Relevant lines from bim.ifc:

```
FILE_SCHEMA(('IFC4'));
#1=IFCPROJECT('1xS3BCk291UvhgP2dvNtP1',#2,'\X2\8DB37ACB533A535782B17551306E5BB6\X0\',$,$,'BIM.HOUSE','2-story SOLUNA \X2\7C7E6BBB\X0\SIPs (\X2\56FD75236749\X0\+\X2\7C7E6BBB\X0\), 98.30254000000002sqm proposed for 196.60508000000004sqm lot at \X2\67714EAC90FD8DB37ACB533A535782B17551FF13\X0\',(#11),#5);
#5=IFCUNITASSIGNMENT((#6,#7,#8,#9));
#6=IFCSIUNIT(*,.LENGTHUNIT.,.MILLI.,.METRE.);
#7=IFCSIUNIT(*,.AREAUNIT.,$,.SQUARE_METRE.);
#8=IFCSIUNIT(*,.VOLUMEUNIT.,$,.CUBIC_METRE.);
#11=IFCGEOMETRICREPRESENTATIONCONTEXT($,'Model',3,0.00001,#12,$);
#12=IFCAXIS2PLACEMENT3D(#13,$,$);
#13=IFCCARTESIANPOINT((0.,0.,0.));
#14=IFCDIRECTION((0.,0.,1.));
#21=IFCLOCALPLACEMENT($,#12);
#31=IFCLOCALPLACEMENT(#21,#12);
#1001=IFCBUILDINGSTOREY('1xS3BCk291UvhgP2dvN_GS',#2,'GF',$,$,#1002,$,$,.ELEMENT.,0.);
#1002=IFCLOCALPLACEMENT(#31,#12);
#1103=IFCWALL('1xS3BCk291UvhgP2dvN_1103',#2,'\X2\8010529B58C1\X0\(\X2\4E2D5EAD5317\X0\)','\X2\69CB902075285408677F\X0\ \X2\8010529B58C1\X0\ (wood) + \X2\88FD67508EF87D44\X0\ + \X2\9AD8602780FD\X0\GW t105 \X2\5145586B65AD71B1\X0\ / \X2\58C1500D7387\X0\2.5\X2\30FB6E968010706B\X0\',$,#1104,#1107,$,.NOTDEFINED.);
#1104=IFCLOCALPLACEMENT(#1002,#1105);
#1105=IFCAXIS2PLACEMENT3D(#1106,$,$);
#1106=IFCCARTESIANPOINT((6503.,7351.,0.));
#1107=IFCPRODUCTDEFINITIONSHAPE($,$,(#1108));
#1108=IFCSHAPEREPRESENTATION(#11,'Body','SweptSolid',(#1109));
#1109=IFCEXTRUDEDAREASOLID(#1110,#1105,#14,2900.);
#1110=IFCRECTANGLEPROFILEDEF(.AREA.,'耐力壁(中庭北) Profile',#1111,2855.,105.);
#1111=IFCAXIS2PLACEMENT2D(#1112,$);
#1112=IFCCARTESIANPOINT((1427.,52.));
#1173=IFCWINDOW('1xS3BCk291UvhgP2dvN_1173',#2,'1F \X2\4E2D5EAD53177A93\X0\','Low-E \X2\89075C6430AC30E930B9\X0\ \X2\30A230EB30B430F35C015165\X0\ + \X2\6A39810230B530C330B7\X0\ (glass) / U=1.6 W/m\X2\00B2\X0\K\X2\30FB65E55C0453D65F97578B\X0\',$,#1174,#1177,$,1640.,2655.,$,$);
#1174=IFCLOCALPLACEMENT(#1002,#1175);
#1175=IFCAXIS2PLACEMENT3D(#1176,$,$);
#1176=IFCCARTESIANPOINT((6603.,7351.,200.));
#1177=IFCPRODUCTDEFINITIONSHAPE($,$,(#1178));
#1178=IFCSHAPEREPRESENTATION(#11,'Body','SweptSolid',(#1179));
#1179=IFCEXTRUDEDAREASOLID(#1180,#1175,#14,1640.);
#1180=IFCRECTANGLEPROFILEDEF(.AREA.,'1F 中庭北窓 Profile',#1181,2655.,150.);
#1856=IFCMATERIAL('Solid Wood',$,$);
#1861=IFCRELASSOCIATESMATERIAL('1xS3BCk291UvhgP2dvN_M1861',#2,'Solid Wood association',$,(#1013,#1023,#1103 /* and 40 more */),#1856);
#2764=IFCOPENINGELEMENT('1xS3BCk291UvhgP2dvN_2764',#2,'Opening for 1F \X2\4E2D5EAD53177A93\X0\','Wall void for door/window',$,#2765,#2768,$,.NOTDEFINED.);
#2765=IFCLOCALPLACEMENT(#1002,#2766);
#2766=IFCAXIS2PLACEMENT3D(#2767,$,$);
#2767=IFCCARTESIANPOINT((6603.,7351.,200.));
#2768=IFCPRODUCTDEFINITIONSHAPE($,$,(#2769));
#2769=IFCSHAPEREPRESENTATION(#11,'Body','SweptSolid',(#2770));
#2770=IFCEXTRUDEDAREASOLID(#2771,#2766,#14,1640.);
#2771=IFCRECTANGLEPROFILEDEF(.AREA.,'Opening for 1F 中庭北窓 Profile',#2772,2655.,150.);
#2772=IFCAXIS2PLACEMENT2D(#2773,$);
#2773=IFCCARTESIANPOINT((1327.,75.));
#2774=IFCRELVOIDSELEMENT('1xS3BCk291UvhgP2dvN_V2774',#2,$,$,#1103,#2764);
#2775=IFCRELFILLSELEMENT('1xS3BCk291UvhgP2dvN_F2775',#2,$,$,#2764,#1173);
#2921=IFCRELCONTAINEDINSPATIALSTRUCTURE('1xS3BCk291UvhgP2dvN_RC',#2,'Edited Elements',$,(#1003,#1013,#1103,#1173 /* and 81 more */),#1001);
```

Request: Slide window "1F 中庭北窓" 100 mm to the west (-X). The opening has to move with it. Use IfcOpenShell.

```python
import ifcopenshell
import ifcopenshell.api.geometry
import ifcopenshell.util.placement
import ifcopenshell.util.unit

model = ifcopenshell.open("bim.ifc")
unit_scale = ifcopenshell.util.unit.calculate_unit_scale(model)

window = model.by_guid("1xS3BCk291UvhgP2dvN_1173")
opening = window.FillsVoids[0].RelatingOpeningElement
wall = opening.VoidsElements[0].RelatingBuildingElement

wall_matrix = ifcopenshell.util.placement.get_local_placement(wall.ObjectPlacement)
shift = wall_matrix[:3, 0] * -0.1 / unit_scale
before = ifcopenshell.util.placement.get_local_placement(window.ObjectPlacement)[:3, 3].copy()

# The window is not placed relative to its opening, so move both.
for product in (opening, window):
    matrix = ifcopenshell.util.placement.get_local_placement(product.ObjectPlacement)
    matrix[:3, 3] += shift
    ifcopenshell.api.geometry.edit_object_placement(model, product=product, matrix=matrix, is_si=False)

after = ifcopenshell.util.placement.get_local_placement(window.ObjectPlacement)[:3, 3]
print("window moved by", (after - before).round(3) + 0.0)

model.write("bim_edited.ifc")
```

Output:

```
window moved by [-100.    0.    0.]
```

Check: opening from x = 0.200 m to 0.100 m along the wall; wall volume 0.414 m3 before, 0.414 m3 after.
